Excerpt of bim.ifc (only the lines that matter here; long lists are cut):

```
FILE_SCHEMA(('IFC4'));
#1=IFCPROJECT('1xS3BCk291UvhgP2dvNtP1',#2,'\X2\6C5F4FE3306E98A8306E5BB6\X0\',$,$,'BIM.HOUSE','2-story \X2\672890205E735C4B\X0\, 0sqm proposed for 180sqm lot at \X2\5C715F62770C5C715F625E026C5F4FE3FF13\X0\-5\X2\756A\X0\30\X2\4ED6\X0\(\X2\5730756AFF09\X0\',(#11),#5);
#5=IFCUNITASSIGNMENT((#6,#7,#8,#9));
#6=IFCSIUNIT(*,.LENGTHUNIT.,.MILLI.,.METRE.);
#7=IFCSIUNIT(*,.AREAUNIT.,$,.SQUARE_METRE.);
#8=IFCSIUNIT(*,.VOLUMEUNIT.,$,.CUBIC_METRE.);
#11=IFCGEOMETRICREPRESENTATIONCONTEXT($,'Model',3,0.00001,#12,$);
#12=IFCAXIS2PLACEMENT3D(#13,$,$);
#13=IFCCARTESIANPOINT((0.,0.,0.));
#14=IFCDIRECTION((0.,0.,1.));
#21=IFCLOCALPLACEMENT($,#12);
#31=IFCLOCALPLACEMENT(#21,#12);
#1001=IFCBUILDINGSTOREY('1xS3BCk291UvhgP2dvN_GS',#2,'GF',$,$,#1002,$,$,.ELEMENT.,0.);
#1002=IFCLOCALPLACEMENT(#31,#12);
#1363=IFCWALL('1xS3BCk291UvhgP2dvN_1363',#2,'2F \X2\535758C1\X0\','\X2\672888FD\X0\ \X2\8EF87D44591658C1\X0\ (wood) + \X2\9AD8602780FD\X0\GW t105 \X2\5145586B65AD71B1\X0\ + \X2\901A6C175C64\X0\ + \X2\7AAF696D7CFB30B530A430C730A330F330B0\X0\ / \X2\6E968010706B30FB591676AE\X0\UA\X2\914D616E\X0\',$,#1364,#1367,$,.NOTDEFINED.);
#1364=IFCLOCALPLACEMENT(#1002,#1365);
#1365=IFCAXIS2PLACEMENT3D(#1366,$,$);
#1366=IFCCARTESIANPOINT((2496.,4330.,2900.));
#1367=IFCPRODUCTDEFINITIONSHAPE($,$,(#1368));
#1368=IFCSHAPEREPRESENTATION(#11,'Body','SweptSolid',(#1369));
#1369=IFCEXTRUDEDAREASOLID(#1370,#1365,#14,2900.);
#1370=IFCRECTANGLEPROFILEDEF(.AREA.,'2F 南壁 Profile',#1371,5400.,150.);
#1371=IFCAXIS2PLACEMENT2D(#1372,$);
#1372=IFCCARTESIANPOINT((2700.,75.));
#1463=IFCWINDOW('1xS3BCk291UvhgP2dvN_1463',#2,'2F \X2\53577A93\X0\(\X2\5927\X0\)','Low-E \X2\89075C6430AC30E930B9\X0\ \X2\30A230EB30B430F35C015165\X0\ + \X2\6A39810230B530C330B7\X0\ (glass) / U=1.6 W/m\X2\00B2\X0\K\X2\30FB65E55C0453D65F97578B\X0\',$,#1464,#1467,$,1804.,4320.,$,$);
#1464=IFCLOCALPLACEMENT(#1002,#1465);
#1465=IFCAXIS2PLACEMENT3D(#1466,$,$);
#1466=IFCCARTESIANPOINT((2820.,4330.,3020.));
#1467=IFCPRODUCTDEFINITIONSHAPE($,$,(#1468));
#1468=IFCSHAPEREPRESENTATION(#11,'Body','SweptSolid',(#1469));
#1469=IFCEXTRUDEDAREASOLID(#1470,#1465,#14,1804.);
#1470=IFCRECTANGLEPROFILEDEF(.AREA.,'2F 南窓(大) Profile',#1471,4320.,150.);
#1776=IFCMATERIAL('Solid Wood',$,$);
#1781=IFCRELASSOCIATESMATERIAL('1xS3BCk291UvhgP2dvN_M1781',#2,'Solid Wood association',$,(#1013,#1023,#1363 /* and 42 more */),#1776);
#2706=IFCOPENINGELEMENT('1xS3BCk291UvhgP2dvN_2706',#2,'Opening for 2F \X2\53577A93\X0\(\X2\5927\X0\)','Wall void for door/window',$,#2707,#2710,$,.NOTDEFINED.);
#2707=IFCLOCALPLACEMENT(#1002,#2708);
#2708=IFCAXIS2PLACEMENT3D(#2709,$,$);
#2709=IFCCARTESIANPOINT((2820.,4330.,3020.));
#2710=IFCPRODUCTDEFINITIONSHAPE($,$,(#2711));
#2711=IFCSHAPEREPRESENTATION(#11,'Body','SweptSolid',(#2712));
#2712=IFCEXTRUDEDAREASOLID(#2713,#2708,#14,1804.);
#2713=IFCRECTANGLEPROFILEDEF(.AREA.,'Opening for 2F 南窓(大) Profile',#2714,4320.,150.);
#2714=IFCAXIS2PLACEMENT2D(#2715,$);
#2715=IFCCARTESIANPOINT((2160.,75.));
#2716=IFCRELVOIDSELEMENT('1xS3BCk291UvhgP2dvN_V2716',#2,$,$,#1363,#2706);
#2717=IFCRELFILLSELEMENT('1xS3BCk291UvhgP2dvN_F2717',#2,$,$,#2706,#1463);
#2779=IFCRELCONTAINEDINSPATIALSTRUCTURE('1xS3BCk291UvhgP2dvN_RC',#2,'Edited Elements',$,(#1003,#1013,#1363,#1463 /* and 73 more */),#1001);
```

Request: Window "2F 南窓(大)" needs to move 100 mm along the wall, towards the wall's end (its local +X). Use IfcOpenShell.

```python
import ifcopenshell
import ifcopenshell.api.geometry
import ifcopenshell.util.placement

model = ifcopenshell.open("bim.ifc")

window = model.by_id(1463)
opening = window.FillsVoids[0].RelatingOpeningElement
wall = opening.VoidsElements[0].RelatingBuildingElement

wall_matrix = ifcopenshell.util.placement.get_local_placement(wall.ObjectPlacement)
shift = wall_matrix[:3, 0] * 100.0
before = ifcopenshell.util.placement.get_local_placement(window.ObjectPlacement)[:3, 3].copy()

# The window is not placed relative to its opening, so move both.
for product in (opening, window):
    matrix = ifcopenshell.util.placement.get_local_placement(product.ObjectPlacement)
    matrix[:3, 3] += shift
    ifcopenshell.api.geometry.edit_object_placement(model, product=product, matrix=matrix, is_si=False)

after = ifcopenshell.util.placement.get_local_placement(window.ObjectPlacement)[:3, 3]
print("window moved by", (after - before).round(3) + 0.0)

model.write("bim_rev.ifc")
```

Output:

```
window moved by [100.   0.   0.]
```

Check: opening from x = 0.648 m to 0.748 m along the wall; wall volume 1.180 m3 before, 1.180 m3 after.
